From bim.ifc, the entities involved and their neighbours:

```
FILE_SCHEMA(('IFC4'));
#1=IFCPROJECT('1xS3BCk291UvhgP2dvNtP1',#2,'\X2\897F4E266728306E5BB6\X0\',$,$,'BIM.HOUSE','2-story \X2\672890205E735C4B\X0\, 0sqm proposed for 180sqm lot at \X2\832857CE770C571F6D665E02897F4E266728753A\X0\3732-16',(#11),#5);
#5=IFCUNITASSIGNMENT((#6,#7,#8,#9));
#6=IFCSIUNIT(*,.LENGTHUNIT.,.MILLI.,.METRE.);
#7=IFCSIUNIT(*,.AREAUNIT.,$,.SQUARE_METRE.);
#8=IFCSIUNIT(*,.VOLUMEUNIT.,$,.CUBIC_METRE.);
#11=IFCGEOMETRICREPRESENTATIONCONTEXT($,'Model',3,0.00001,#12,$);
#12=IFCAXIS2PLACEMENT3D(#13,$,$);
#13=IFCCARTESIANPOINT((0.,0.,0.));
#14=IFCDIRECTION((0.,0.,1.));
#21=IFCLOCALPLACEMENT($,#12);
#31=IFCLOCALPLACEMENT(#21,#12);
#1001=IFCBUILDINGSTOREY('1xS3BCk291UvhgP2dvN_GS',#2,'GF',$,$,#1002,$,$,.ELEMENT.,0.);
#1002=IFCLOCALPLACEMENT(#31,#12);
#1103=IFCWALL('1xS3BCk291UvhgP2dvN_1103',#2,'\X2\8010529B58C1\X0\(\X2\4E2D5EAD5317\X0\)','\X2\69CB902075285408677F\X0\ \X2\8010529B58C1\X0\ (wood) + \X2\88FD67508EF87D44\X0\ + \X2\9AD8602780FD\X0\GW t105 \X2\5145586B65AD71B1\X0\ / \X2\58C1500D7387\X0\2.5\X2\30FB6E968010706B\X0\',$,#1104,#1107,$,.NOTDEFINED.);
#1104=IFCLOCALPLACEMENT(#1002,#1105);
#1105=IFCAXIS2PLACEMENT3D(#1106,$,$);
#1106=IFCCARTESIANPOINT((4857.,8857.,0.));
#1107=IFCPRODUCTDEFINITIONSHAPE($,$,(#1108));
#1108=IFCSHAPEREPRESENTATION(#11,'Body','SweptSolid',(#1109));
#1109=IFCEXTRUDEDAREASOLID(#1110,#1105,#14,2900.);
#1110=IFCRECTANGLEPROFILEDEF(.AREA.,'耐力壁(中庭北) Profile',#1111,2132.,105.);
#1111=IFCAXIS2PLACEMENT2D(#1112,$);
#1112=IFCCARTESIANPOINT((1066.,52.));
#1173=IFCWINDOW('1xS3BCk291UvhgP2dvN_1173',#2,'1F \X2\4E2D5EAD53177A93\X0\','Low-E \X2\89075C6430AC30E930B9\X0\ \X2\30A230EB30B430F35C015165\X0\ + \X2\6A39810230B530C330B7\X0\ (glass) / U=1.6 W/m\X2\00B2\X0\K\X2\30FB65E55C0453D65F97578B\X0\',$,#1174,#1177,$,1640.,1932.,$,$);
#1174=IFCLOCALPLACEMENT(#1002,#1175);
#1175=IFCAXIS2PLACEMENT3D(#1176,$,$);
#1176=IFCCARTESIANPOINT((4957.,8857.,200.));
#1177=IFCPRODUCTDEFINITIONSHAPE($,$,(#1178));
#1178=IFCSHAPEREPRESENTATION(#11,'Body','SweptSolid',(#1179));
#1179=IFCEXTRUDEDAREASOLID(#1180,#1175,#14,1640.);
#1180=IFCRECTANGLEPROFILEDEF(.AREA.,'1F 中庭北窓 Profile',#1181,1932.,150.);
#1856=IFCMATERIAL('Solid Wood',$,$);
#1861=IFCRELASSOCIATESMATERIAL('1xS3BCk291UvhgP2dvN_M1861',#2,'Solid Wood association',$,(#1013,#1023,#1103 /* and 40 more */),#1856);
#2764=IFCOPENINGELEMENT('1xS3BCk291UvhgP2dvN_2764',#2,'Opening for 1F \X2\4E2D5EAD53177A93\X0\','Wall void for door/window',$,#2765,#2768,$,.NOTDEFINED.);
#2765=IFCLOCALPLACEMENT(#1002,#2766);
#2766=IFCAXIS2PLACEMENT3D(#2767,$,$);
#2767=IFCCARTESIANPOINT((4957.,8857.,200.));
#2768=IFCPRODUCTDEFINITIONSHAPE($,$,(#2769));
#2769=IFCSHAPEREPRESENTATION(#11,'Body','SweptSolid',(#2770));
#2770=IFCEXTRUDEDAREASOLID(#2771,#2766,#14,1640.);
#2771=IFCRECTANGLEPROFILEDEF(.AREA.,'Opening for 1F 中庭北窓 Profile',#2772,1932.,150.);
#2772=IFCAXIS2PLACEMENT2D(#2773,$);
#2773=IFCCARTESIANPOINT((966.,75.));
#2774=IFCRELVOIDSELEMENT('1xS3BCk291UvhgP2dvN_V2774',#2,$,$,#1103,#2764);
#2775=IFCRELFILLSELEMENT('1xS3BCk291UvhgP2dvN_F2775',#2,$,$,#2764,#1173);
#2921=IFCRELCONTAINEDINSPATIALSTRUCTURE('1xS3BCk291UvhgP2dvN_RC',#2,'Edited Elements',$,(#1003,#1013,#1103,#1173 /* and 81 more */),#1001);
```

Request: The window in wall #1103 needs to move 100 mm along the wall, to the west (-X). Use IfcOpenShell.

```python
import ifcopenshell
import ifcopenshell.api.geometry
import ifcopenshell.util.placement
import ifcopenshell.util.unit

model = ifcopenshell.open("bim.ifc")
unit_scale = ifcopenshell.util.unit.calculate_unit_scale(model)

window = model.by_id(1173)
opening = window.FillsVoids[0].RelatingOpeningElement
wall = opening.VoidsElements[0].RelatingBuildingElement

wall_matrix = ifcopenshell.util.placement.get_local_placement(wall.ObjectPlacement)
shift = wall_matrix[:3, 0] * -0.1 / unit_scale
before = ifcopenshell.util.placement.get_local_placement(window.ObjectPlacement)[:3, 3].copy()

# The window is not placed relative to its opening, so move both.
for product in (opening, window):
    matrix = ifcopenshell.util.placement.get_local_placement(product.ObjectPlacement)
    matrix[:3, 3] += shift
    ifcopenshell.api.geometry.edit_object_placement(model, product=product, matrix=matrix, is_si=False)

after = ifcopenshell.util.placement.get_local_placement(window.ObjectPlacement)[:3, 3]
print("window moved by", (after - before).round(3) + 0.0)

model.write("bim_v2.ifc")
```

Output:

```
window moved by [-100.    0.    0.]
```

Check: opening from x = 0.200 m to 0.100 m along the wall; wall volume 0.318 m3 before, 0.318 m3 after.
